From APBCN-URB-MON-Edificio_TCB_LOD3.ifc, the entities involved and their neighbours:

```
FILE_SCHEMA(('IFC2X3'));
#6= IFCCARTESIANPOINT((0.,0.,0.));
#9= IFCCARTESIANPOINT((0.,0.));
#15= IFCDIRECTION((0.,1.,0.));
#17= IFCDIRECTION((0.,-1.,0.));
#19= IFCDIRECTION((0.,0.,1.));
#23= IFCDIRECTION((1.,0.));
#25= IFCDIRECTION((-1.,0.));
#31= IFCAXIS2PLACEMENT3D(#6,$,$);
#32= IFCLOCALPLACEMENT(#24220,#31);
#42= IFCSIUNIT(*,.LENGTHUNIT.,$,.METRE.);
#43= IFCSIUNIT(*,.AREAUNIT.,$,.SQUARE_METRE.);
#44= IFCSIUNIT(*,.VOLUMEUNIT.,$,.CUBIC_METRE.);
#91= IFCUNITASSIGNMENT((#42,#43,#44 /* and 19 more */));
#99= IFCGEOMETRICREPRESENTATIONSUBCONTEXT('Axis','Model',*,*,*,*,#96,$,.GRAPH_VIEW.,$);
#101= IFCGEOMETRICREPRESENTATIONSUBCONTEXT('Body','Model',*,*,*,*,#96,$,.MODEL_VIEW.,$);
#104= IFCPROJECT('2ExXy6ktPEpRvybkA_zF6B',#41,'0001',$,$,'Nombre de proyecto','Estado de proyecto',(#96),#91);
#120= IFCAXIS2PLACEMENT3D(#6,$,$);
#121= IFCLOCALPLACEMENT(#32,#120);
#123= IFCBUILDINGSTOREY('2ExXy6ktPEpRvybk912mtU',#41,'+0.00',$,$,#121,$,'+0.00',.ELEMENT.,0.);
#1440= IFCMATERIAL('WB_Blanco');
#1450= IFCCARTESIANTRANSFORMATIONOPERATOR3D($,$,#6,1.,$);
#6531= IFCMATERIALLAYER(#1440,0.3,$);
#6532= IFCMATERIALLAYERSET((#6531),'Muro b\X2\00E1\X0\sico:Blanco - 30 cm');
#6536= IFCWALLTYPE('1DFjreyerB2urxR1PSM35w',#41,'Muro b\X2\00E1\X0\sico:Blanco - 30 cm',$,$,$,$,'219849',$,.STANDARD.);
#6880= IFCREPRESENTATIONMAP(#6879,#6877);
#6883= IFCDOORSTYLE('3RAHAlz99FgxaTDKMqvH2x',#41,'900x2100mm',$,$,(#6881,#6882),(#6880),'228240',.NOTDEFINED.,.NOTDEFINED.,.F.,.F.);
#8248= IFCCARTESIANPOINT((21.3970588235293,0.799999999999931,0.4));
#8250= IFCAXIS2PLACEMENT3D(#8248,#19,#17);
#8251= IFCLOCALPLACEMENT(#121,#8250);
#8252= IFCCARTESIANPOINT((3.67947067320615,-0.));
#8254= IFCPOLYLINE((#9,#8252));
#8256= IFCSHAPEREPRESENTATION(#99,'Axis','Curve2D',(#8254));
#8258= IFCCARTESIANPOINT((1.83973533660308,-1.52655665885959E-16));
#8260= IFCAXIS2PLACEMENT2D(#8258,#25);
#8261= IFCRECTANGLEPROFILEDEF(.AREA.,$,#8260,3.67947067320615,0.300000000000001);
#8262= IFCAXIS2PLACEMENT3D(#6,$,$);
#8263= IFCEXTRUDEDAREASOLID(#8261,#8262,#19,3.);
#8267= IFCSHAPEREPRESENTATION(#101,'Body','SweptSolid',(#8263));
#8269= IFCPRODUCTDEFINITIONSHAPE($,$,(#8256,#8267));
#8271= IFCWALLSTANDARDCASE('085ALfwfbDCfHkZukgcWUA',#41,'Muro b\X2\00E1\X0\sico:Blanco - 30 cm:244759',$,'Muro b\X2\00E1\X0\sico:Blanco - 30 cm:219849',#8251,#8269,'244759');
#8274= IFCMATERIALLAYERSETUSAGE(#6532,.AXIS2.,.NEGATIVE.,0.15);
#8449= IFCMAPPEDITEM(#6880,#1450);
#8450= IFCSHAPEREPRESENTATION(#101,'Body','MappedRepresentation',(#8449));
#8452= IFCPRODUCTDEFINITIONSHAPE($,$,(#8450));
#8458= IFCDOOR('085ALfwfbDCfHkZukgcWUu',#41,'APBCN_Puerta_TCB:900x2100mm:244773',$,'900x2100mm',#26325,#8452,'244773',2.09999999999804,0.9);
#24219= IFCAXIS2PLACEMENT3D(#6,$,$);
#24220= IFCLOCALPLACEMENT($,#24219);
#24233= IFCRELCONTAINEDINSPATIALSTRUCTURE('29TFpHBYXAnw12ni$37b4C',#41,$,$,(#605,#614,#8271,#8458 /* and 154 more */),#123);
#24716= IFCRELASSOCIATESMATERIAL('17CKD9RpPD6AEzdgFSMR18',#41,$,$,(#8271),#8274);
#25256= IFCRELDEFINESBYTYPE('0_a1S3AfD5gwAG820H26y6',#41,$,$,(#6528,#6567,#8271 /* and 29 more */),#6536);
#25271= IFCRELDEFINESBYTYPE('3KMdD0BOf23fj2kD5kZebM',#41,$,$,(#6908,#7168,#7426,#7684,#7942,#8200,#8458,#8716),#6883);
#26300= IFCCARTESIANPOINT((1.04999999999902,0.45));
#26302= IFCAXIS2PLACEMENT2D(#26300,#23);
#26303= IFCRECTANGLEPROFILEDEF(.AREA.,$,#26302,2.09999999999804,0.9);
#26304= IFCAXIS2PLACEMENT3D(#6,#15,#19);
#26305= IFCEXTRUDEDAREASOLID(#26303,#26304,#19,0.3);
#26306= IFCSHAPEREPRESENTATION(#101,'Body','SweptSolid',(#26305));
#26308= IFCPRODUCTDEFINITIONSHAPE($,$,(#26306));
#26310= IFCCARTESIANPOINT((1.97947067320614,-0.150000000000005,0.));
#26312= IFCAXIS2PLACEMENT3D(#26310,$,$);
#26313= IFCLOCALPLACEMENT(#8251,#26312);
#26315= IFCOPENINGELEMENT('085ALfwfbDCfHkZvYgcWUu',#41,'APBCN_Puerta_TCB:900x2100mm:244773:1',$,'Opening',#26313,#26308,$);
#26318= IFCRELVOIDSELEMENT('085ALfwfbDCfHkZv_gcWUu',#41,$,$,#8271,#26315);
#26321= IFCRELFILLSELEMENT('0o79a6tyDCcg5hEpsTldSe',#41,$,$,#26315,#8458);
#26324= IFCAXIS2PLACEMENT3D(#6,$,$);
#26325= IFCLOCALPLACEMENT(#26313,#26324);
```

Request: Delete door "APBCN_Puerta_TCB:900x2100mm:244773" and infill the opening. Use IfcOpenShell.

```python
import ifcopenshell
import ifcopenshell.api.feature
import ifcopenshell.api.root
import ifcopenshell.geom
import ifcopenshell.util.shape

model = ifcopenshell.open("APBCN-URB-MON-Edificio_TCB_LOD3.ifc")
settings = ifcopenshell.geom.settings()


def volume(element):
    """Net volume in cubic metres, openings subtracted."""
    shape = ifcopenshell.geom.create_shape(settings, element)
    return ifcopenshell.util.shape.get_volume(shape.geometry)


door = model.by_guid("085ALfwfbDCfHkZukgcWUu")
opening = door.FillsVoids[0].RelatingOpeningElement
wall = opening.VoidsElements[0].RelatingBuildingElement
before = volume(wall)

ifcopenshell.api.root.remove_product(model, product=door)
ifcopenshell.api.feature.remove_feature(model, feature=opening)

after = volume(wall)

print(f"wall volume {before:.3f} -> {after:.3f} m3")

model.write("APBCN-URB-MON-Edificio_TCB_LOD3_v2.ifc")
```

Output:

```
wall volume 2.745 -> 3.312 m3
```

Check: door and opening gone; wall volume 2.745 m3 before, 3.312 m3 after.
